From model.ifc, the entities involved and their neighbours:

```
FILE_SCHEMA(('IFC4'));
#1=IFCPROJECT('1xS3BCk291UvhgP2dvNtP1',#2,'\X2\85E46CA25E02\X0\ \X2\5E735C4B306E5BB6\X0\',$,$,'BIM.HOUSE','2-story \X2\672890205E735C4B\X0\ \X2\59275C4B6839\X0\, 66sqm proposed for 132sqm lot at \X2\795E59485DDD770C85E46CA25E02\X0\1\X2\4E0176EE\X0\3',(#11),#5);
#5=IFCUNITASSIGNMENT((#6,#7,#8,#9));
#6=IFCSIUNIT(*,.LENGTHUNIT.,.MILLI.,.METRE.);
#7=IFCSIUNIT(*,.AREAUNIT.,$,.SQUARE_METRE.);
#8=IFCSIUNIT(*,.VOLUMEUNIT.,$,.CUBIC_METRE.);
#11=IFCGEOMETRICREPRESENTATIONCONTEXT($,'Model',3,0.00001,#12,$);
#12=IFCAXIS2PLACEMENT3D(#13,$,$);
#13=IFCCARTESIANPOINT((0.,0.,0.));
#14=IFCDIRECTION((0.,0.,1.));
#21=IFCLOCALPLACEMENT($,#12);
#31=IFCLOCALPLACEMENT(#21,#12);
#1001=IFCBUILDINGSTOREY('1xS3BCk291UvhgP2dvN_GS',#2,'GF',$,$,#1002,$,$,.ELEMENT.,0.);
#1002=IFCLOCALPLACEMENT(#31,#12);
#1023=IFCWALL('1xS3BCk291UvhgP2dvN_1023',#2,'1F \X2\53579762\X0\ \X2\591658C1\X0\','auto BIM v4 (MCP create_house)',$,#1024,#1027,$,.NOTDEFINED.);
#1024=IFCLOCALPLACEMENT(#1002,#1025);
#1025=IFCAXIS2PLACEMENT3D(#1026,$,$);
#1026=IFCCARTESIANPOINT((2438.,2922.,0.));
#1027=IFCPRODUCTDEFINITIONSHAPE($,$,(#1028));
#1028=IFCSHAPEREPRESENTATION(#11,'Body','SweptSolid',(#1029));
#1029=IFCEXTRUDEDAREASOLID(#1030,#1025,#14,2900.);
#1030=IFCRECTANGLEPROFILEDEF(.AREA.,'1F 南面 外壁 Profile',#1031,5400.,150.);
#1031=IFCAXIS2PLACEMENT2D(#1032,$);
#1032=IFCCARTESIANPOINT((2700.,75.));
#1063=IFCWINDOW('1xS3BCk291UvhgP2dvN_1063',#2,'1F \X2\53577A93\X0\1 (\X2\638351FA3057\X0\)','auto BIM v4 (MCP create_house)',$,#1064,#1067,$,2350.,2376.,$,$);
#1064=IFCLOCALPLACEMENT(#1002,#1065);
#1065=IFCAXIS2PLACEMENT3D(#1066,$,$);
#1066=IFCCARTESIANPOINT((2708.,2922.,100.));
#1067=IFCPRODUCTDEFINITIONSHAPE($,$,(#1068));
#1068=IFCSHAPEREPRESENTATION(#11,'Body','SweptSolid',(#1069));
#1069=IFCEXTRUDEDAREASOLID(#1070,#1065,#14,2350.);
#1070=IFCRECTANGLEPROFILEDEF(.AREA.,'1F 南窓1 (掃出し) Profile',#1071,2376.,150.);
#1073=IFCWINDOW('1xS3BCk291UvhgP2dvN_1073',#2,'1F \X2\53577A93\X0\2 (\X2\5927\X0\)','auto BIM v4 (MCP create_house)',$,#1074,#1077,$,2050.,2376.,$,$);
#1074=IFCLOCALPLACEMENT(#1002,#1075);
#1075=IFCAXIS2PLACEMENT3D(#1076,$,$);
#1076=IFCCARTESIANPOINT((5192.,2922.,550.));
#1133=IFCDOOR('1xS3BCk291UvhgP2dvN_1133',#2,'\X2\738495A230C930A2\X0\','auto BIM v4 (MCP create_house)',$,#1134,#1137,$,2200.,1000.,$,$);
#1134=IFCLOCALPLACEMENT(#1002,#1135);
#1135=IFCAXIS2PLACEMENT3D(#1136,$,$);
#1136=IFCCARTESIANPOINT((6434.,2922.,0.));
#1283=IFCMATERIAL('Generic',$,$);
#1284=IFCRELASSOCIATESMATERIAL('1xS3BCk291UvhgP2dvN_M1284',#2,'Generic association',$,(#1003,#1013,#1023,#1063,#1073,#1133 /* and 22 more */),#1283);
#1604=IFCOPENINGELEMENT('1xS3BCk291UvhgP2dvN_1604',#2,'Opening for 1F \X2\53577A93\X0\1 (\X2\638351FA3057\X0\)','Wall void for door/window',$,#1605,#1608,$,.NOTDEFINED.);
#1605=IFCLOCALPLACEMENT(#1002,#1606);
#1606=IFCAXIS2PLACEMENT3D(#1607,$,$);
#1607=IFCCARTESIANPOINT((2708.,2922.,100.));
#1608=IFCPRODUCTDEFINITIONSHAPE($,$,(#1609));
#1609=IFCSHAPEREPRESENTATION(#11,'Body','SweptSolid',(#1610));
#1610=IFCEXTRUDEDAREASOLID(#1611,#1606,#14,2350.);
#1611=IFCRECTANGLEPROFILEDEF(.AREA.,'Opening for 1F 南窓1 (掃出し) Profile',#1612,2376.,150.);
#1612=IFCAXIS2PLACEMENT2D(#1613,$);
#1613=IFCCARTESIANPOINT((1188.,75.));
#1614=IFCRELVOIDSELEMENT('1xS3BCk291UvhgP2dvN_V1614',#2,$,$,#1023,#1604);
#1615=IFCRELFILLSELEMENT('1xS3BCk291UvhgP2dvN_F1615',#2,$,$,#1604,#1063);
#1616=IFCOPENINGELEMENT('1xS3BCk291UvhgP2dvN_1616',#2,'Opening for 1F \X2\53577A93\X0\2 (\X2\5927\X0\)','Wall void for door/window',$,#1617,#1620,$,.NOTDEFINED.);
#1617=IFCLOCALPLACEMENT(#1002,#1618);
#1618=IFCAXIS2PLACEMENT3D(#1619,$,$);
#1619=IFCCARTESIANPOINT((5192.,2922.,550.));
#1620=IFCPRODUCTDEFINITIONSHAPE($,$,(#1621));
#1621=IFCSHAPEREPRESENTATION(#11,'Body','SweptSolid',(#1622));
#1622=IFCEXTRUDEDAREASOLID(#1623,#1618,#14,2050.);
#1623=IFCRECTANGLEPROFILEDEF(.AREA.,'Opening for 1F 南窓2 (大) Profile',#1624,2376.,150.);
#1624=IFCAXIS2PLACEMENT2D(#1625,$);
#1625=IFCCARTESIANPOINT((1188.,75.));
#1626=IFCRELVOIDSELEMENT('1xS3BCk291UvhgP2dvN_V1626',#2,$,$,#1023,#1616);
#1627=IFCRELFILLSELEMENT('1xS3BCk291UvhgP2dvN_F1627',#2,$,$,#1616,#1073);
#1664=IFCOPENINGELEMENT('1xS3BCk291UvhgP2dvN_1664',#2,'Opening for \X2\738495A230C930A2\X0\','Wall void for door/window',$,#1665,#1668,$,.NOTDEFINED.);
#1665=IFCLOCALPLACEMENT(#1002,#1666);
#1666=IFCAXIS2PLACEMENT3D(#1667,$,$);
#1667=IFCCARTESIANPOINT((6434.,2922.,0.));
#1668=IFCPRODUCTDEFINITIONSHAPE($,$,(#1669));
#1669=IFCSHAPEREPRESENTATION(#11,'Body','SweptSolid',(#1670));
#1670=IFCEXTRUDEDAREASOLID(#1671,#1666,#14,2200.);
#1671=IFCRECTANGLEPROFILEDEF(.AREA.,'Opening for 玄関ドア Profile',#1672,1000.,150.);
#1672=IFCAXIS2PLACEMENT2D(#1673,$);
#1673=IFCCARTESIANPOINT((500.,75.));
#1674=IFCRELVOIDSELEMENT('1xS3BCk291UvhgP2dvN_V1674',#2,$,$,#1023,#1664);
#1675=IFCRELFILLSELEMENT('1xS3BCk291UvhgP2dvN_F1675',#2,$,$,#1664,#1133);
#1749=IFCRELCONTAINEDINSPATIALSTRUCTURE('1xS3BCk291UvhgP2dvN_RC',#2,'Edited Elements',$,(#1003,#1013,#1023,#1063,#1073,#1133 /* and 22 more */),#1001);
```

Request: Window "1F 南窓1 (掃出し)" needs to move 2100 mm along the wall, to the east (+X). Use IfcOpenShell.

```python
import ifcopenshell
import ifcopenshell.api.geometry
import ifcopenshell.util.placement
import ifcopenshell.util.unit

model = ifcopenshell.open("model.ifc")
unit_scale = ifcopenshell.util.unit.calculate_unit_scale(model)

window = model.by_guid("1xS3BCk291UvhgP2dvN_1063")
opening = window.FillsVoids[0].RelatingOpeningElement
wall = opening.VoidsElements[0].RelatingBuildingElement

wall_matrix = ifcopenshell.util.placement.get_local_placement(wall.ObjectPlacement)
shift = wall_matrix[:3, 0] * 2.1 / unit_scale
before = ifcopenshell.util.placement.get_local_placement(window.ObjectPlacement)[:3, 3].copy()

# The window is not placed relative to its opening, so move both.
for product in (opening, window):
    matrix = ifcopenshell.util.placement.get_local_placement(product.ObjectPlacement)
    matrix[:3, 3] += shift
    ifcopenshell.api.geometry.edit_object_placement(model, product=product, matrix=matrix, is_si=False)

after = ifcopenshell.util.placement.get_local_placement(window.ObjectPlacement)[:3, 3]
print("window moved by", (after - before).round(3) + 0.0)

model.write("model_edited.ifc")
```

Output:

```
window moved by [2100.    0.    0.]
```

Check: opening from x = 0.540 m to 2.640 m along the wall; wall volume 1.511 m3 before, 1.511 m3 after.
